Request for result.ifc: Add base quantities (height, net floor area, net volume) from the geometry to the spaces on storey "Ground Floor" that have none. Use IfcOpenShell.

First a look at what the model holds.

```python
import ifcopenshell
import ifcopenshell.util.element
import ifcopenshell.util.unit

model = ifcopenshell.open("result.ifc")
print(model.schema)
for unit_type in ("LENGTHUNIT", "AREAUNIT", "VOLUMEUNIT"):
    print(unit_type, ifcopenshell.util.unit.calculate_unit_scale(model, unit_type))
storey = next(s for s in model.by_type("IfcBuildingStorey") if s.Name == "Ground Floor")
spaces = [e for e in ifcopenshell.util.element.get_decomposition(storey) if e.is_a("IfcSpace")]
for e in sorted(spaces, key=lambda e: e.id()):
    print(e.id(), e.is_a(), e.Name, list(ifcopenshell.util.element.get_psets(e, qtos_only=True)), sep=" | ")
```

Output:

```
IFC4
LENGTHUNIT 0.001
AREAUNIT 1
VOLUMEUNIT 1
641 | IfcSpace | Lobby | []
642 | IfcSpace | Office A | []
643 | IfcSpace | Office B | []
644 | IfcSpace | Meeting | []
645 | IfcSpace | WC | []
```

```python
import ifcopenshell
import ifcopenshell.api.pset
import ifcopenshell.geom
import ifcopenshell.util.element
import ifcopenshell.util.shape
import ifcopenshell.util.unit

model = ifcopenshell.open("result.ifc")
unit_scale = ifcopenshell.util.unit.calculate_unit_scale(model)
area_scale = ifcopenshell.util.unit.calculate_unit_scale(model, "AREAUNIT")
volume_scale = ifcopenshell.util.unit.calculate_unit_scale(model, "VOLUMEUNIT")
settings = ifcopenshell.geom.settings()

storey = next(s for s in model.by_type("IfcBuildingStorey") if s.Name == "Ground Floor")
spaces = [e for e in ifcopenshell.util.element.get_decomposition(storey) if e.is_a("IfcSpace")]

for e in sorted(spaces, key=lambda e: e.id()):
    if ifcopenshell.util.element.get_psets(e, qtos_only=True, should_inherit=False):
        continue
    # Geometry comes back in metres, in the element's own axes.
    shape = ifcopenshell.geom.create_shape(settings, e)
    values = {
        "Height": ifcopenshell.util.shape.get_z(shape.geometry) / unit_scale,
        "NetFloorArea": ifcopenshell.util.shape.get_footprint_area(shape.geometry) / area_scale,
        "NetVolume": ifcopenshell.util.shape.get_volume(shape.geometry) / volume_scale,
    }
    qto = ifcopenshell.api.pset.add_qto(model, product=e, name="Qto_SpaceBaseQuantities")
    ifcopenshell.api.pset.edit_qto(model, qto=qto, properties=values)
    print(e.id(), {k: round(v, 3) for k, v in values.items()})

model.write("result_edited.ifc")
```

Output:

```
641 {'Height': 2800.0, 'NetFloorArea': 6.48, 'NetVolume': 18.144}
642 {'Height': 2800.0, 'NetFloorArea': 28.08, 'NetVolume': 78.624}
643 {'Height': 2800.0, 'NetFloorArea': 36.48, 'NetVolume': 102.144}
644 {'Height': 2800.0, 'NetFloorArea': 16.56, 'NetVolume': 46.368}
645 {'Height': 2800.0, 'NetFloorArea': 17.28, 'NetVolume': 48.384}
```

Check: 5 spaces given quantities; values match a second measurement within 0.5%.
